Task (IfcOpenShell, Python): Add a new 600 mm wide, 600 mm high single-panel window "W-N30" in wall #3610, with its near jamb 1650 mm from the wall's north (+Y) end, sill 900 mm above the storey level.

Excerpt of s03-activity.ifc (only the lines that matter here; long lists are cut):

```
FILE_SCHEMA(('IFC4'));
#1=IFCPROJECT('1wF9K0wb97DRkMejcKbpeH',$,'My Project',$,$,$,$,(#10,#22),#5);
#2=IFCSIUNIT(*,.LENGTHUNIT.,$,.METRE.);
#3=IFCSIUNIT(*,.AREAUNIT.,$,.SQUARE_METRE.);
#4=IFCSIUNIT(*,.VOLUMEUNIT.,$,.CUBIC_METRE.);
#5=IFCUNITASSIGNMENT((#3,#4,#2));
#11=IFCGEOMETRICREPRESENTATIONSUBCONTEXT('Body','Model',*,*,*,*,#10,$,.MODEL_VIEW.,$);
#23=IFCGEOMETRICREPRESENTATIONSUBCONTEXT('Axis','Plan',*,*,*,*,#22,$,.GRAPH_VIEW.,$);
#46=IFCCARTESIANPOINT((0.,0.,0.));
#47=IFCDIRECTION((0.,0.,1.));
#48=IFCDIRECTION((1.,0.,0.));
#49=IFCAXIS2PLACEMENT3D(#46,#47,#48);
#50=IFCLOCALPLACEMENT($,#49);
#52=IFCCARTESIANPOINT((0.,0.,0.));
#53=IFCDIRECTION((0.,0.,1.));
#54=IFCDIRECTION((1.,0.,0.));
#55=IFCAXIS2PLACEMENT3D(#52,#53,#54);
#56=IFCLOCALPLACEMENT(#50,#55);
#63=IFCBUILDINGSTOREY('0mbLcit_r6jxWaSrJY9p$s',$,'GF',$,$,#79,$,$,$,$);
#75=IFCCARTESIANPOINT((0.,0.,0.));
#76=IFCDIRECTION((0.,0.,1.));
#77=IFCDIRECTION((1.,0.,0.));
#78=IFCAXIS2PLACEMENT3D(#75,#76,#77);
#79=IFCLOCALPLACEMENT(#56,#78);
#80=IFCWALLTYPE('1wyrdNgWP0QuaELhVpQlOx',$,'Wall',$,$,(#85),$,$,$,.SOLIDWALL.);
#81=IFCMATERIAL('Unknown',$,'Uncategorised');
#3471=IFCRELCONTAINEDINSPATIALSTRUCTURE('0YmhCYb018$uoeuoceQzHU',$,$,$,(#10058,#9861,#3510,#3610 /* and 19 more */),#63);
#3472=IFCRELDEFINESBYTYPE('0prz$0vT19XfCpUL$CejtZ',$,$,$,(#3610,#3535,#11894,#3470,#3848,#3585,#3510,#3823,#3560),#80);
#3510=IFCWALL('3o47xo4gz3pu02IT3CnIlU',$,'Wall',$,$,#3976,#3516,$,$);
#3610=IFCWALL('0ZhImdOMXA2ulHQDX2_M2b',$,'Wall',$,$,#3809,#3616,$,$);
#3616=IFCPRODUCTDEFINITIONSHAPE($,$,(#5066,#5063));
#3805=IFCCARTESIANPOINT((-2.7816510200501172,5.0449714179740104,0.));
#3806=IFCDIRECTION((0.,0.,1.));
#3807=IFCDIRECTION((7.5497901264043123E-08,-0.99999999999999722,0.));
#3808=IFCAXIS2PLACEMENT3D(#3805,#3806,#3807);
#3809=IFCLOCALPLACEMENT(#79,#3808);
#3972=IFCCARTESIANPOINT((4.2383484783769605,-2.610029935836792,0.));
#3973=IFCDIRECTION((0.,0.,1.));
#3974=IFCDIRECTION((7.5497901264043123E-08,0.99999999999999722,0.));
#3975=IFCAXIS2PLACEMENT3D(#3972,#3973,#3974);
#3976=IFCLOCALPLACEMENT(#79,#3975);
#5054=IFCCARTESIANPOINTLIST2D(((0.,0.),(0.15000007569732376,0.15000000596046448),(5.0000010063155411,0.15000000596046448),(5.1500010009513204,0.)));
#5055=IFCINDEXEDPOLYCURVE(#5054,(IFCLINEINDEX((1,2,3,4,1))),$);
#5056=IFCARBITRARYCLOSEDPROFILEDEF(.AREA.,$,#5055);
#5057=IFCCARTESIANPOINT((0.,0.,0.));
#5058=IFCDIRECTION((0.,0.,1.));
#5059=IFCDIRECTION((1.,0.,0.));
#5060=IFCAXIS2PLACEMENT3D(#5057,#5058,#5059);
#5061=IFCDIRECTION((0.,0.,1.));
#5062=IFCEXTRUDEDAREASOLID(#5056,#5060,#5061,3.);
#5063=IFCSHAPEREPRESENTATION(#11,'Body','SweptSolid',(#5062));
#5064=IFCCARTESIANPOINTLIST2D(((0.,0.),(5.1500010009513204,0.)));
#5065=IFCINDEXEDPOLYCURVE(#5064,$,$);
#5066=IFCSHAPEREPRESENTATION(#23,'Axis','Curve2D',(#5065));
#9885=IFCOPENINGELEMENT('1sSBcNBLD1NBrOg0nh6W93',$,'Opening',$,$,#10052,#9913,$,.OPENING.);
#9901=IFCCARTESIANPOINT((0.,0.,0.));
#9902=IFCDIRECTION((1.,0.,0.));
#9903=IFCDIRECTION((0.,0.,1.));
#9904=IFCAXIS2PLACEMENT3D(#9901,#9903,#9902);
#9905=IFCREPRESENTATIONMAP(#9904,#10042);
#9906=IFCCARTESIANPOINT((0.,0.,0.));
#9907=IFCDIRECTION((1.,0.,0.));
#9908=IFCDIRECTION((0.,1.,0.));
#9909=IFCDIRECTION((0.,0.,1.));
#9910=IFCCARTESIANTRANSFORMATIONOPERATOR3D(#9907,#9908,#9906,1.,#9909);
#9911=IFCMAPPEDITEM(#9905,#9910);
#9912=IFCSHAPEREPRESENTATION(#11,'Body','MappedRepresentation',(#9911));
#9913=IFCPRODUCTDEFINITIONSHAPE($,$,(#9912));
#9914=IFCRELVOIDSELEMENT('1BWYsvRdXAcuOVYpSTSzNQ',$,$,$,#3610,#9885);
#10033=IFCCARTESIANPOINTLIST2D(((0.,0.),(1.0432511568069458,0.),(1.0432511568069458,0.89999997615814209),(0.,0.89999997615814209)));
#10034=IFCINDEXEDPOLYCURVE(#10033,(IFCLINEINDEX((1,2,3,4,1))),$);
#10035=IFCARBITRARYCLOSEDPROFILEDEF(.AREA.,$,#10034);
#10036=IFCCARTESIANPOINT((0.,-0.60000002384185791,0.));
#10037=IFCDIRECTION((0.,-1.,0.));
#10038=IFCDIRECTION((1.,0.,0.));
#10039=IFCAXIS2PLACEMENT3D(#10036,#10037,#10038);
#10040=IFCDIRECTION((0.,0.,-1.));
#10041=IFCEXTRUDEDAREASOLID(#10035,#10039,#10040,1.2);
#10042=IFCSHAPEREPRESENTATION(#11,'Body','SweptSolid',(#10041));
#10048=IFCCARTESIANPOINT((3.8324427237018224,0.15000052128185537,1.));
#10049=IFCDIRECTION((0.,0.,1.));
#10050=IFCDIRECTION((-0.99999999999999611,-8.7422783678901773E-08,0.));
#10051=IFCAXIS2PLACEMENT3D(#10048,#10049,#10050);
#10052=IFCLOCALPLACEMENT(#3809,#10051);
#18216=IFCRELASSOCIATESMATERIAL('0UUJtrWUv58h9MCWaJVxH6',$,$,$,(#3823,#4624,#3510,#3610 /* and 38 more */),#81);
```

```python
import numpy as np
import ifcopenshell
import ifcopenshell.api.feature
import ifcopenshell.api.geometry
import ifcopenshell.api.root
import ifcopenshell.api.spatial
import ifcopenshell.geom
import ifcopenshell.util.element
import ifcopenshell.util.placement
import ifcopenshell.util.representation
import ifcopenshell.util.shape
import ifcopenshell.util.unit

model = ifcopenshell.open("s03-activity.ifc")
unit_scale = ifcopenshell.util.unit.calculate_unit_scale(model)
settings = ifcopenshell.geom.settings()


def volume(element):
    """Net volume in cubic metres, openings subtracted."""
    shape = ifcopenshell.geom.create_shape(settings, element)
    return ifcopenshell.util.shape.get_volume(shape.geometry)


wall = model.by_guid("0ZhImdOMXA2ulHQDX2_M2b")
storey = ifcopenshell.util.element.get_container(wall, ifc_class="IfcBuildingStorey")
context = ifcopenshell.util.representation.get_context(model, "Model", "Body", "MODEL_VIEW")
before = volume(wall)

width, height, from_end, sill = 0.6, 0.6, 1.65, 0.9  # metres

# The wall runs along its own X axis, and the end named is its -X end.
wall_shape = ifcopenshell.geom.create_shape(settings, wall)
x, y, z = ifcopenshell.util.shape.get_vertices(wall_shape.geometry).T
start = x.min() + from_end
face, thickness = float(y.min()), float(y.max() - y.min())
wall_matrix = ifcopenshell.util.placement.get_local_placement(wall.ObjectPlacement)
level = ifcopenshell.util.placement.get_local_placement(storey.ObjectPlacement)[2, 3]


def in_wall(x, y):
    """Placement at x, y metres in the wall's axes, at sill height."""
    matrix = wall_matrix.copy()
    matrix[:, 3] = wall_matrix @ np.array([x / unit_scale, y / unit_scale, 0.0, 1.0])
    matrix[2, 3] = level + sill / unit_scale
    return matrix


# Opening: a box that overshoots both wall faces by 50 mm.
opening = ifcopenshell.api.root.create_entity(model, ifc_class="IfcOpeningElement", predefined_type="OPENING")
box = ifcopenshell.api.geometry.add_wall_representation(
    model, context=context, length=width, height=height, thickness=thickness + 0.1
)
ifcopenshell.api.geometry.assign_representation(model, product=opening, representation=box)
ifcopenshell.api.geometry.edit_object_placement(model, product=opening, matrix=in_wall(start, face - 0.05), is_si=False)
ifcopenshell.api.feature.add_feature(model, feature=opening, element=wall)

window = ifcopenshell.api.root.create_entity(model, ifc_class="IfcWindow", name="W-N30", predefined_type="WINDOW")
window.OverallWidth, window.OverallHeight = width / unit_scale, height / unit_scale
window.PartitioningType = "SINGLE_PANEL"
body = ifcopenshell.api.geometry.add_window_representation(
    model,
    context=context,
    overall_width=window.OverallWidth,
    overall_height=window.OverallHeight,
    partition_type="SINGLE_PANEL",
)
ifcopenshell.api.geometry.assign_representation(model, product=window, representation=body)
ifcopenshell.api.spatial.assign_container(model, products=[window], relating_structure=storey)
ifcopenshell.api.feature.add_filling(model, opening=opening, element=window)

# Centre the window in the wall's thickness.
ifcopenshell.api.geometry.edit_object_placement(model, product=window, matrix=in_wall(start, face), is_si=False)
window_shape = ifcopenshell.geom.create_shape(settings, window)
depth = ifcopenshell.util.shape.get_vertices(window_shape.geometry)[:, 1]
offset = face + thickness / 2 - (depth.min() + depth.max()) / 2
ifcopenshell.api.geometry.edit_object_placement(model, product=window, matrix=in_wall(start, offset), is_si=False)

after = volume(wall)

print(f"wall volume {before:.3f} -> {after:.3f} m3")

model.write("s03-activity_rev.ifc")
```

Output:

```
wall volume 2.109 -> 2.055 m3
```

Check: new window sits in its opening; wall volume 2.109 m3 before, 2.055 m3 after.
